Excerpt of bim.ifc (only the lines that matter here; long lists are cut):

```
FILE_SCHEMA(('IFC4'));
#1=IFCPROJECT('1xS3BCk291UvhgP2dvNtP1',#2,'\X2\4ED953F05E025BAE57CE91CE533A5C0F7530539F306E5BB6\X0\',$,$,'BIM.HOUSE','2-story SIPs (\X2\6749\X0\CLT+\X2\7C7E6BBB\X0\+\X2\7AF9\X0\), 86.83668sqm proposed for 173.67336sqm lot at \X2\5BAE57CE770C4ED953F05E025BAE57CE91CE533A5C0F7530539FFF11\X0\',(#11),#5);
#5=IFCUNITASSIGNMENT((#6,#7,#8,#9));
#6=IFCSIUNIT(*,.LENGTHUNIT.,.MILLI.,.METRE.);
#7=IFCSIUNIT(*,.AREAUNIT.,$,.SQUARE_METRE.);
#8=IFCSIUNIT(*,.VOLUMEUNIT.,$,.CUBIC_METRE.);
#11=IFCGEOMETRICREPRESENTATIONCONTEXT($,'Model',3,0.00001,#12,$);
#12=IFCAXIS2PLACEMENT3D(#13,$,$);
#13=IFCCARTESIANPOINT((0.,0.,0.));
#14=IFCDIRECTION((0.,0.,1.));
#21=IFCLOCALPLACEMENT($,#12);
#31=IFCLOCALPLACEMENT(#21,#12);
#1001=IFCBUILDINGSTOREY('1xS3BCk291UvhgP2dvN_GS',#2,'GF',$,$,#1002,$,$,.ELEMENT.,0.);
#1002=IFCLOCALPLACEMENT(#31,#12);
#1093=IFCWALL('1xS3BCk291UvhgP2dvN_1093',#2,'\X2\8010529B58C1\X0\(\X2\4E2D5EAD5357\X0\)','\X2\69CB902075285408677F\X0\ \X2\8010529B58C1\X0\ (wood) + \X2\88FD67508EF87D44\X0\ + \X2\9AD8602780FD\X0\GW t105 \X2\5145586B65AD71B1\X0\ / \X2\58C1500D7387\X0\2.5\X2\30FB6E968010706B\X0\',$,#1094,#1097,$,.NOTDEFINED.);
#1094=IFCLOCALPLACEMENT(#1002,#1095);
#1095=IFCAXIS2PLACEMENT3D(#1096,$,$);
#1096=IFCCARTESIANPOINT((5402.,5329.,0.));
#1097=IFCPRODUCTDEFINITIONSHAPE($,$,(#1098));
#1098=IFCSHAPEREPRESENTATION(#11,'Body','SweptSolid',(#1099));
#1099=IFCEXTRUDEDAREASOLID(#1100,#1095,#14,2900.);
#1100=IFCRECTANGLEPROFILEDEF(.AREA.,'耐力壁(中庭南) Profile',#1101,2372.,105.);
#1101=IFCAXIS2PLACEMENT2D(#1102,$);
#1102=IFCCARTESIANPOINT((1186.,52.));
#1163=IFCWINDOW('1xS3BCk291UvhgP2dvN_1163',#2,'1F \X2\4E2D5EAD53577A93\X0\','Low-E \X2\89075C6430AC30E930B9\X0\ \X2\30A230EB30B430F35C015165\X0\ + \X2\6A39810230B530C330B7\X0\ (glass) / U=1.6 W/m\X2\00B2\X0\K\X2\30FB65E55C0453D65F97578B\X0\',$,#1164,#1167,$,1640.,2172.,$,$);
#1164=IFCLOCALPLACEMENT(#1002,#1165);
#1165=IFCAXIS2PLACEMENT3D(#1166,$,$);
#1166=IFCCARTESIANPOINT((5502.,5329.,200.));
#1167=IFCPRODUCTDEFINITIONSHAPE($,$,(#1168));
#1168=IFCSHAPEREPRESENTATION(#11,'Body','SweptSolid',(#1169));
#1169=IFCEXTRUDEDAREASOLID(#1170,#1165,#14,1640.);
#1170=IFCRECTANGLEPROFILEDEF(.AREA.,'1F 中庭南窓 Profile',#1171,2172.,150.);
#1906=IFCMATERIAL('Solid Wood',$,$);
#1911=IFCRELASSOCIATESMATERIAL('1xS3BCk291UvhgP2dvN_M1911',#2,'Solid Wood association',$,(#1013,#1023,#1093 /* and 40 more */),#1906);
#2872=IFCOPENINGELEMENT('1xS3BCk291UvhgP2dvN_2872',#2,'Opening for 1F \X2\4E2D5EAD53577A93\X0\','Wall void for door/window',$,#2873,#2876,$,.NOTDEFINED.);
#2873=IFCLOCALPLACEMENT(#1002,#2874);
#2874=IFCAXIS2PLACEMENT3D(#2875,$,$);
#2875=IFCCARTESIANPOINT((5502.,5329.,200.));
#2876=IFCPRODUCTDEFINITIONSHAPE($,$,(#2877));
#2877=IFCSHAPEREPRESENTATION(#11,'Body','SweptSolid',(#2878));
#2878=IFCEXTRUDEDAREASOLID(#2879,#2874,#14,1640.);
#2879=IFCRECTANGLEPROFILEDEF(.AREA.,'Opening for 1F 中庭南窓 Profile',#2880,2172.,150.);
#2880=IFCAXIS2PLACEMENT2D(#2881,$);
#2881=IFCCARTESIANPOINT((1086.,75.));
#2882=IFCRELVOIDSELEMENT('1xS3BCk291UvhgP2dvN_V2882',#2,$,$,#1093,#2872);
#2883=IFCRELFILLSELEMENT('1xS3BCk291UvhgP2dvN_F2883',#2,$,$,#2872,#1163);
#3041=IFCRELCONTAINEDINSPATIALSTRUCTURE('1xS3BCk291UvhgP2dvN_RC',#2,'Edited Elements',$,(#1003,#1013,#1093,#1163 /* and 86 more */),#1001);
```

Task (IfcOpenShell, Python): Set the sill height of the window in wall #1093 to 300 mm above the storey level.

```python
import numpy as np
import ifcopenshell
import ifcopenshell.api.geometry
import ifcopenshell.geom
import ifcopenshell.util.element
import ifcopenshell.util.placement
import ifcopenshell.util.shape
import ifcopenshell.util.unit

model = ifcopenshell.open("bim.ifc")
unit_scale = ifcopenshell.util.unit.calculate_unit_scale(model)

window = model.by_id(1163)
opening = window.FillsVoids[0].RelatingOpeningElement
storey = ifcopenshell.util.element.get_container(window, ifc_class="IfcBuildingStorey")
level = ifcopenshell.util.placement.get_local_placement(storey.ObjectPlacement)[2, 3]

# The opening's origin need not be at the sill, so measure its lowest point.
shape = ifcopenshell.geom.create_shape(ifcopenshell.geom.settings(), opening)
bottom = ifcopenshell.util.shape.get_shape_bottom_elevation(shape, shape.geometry) / unit_scale
dz = level + 0.3 / unit_scale - bottom

shift = np.array([0.0, 0.0, dz])
# The window is not placed relative to its opening, so move both.
for product in (opening, window):
    matrix = ifcopenshell.util.placement.get_local_placement(product.ObjectPlacement)
    matrix[:3, 3] += shift
    ifcopenshell.api.geometry.edit_object_placement(model, product=product, matrix=matrix, is_si=False)

print(f"moved by {dz * unit_scale:+.3f} m")

model.write("bim_updated.ifc")
```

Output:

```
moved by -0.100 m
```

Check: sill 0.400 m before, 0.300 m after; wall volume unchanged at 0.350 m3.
